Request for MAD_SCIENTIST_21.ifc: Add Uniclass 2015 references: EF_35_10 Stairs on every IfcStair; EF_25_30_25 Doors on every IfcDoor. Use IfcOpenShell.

First a look at what the model holds.

```python
import ifcopenshell

model = ifcopenshell.open("MAD_SCIENTIST_21.ifc")
print(model.schema)
print("classifications:", [c.Name for c in model.by_type("IfcClassification")])
for ifc_class in ("IfcDoor", "IfcRoof", "IfcStair", "IfcWall", "IfcWindow"):
    print(ifc_class, len(model.by_type(ifc_class)))
```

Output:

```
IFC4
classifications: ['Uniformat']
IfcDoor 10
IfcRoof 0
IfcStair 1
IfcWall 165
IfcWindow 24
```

```python
import ifcopenshell
import ifcopenshell.api.classification

model = ifcopenshell.open("MAD_SCIENTIST_21.ifc")

system = ifcopenshell.api.classification.add_classification(model, classification="Uniclass 2015")

codes = {
    "IfcStair": ("EF_35_10", "Stairs"),
    "IfcDoor": ("EF_25_30_25", "Doors"),
}
for ifc_class, (code, name) in codes.items():
    products = model.by_type(ifc_class)
    ifcopenshell.api.classification.add_reference(
        model, products=products, classification=system, identification=code, name=name
    )
    print(code, len(products))

model.write("MAD_SCIENTIST_21-out.ifc")
```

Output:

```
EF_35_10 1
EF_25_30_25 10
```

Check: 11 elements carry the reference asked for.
